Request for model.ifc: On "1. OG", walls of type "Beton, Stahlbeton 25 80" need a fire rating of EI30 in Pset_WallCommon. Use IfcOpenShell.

First a look at what the model holds.

```python
import ifcopenshell
import ifcopenshell.util.element

model = ifcopenshell.open("model.ifc")
print(model.schema)
storey = next(s for s in model.by_type("IfcBuildingStorey") if s.Name == "1. OG")
walls = [e for e in ifcopenshell.util.element.get_decomposition(storey) if e.is_a("IfcWall")]
seen = {}
for e in walls:
    element_type = ifcopenshell.util.element.get_type(e)
    key = (element_type.Name if element_type != e and element_type else None, ifcopenshell.util.element.get_pset(e, "Pset_WallCommon", "FireRating"))
    seen[key] = seen.get(key, 0) + 1
for (name, value), count in sorted(seen.items(), key=str):
    print(count, "x", name, "|", value)
```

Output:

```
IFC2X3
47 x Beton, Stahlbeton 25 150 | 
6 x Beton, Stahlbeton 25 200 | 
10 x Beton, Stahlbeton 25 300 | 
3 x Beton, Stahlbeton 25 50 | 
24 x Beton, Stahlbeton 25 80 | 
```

```python
import ifcopenshell
import ifcopenshell.api.pset
import ifcopenshell.util.element

model = ifcopenshell.open("model.ifc")

storey = next(s for s in model.by_type("IfcBuildingStorey") if s.Name == "1. OG")
walls = [e for e in ifcopenshell.util.element.get_decomposition(storey) if e.is_a("IfcWall")]

count = 0
for e in walls:
    element_type = ifcopenshell.util.element.get_type(e)
    if element_type in (None, e) or element_type.Name != "Beton, Stahlbeton 25 80":
        continue
    # add_pset returns the element's existing set when there is one.
    pset = ifcopenshell.api.pset.add_pset(model, product=e, name="Pset_WallCommon")
    ifcopenshell.api.pset.edit_pset(model, pset=pset, properties={"FireRating": "EI30"})
    count += 1

print(count, "walls updated")

model.write("model_edited.ifc")
```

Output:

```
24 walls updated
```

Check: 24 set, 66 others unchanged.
